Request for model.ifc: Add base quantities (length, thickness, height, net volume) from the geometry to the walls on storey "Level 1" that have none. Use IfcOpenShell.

First a look at what the model holds.

```python
import ifcopenshell
import ifcopenshell.util.element
import ifcopenshell.util.unit

model = ifcopenshell.open("model.ifc")
print(model.schema)
for unit_type in ("LENGTHUNIT", "AREAUNIT", "VOLUMEUNIT"):
    print(unit_type, ifcopenshell.util.unit.calculate_unit_scale(model, unit_type))
storey = next(s for s in model.by_type("IfcBuildingStorey") if s.Name == "Level 1")
walls = [e for e in ifcopenshell.util.element.get_decomposition(storey) if e.is_a("IfcWall")]
for e in sorted(walls, key=lambda e: e.id()):
    print(e.id(), e.is_a(), e.Name, list(ifcopenshell.util.element.get_psets(e, qtos_only=True)), sep=" | ")
```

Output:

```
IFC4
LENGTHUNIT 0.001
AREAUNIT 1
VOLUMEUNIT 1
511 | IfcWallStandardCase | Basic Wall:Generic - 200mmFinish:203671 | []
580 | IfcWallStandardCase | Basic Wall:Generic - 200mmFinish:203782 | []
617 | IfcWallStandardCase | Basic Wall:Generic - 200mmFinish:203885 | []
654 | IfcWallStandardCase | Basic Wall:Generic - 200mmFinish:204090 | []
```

```python
import ifcopenshell
import ifcopenshell.api.pset
import ifcopenshell.geom
import ifcopenshell.util.element
import ifcopenshell.util.shape
import ifcopenshell.util.unit

model = ifcopenshell.open("model.ifc")
unit_scale = ifcopenshell.util.unit.calculate_unit_scale(model)
volume_scale = ifcopenshell.util.unit.calculate_unit_scale(model, "VOLUMEUNIT")
settings = ifcopenshell.geom.settings()

storey = next(s for s in model.by_type("IfcBuildingStorey") if s.Name == "Level 1")
walls = [e for e in ifcopenshell.util.element.get_decomposition(storey) if e.is_a("IfcWall")]

for e in sorted(walls, key=lambda e: e.id()):
    if ifcopenshell.util.element.get_psets(e, qtos_only=True, should_inherit=False):
        continue
    # Geometry comes back in metres, in the element's own axes.
    shape = ifcopenshell.geom.create_shape(settings, e)
    values = {
        "Length": ifcopenshell.util.shape.get_x(shape.geometry) / unit_scale,
        "Width": ifcopenshell.util.shape.get_y(shape.geometry) / unit_scale,
        "Height": ifcopenshell.util.shape.get_z(shape.geometry) / unit_scale,
        "NetVolume": ifcopenshell.util.shape.get_volume(shape.geometry) / volume_scale,
    }
    qto = ifcopenshell.api.pset.add_qto(model, product=e, name="Qto_WallBaseQuantities")
    ifcopenshell.api.pset.edit_qto(model, qto=qto, properties=values)
    print(e.id(), {k: round(v, 3) for k, v in values.items()})

model.write("model_updated.ifc")
```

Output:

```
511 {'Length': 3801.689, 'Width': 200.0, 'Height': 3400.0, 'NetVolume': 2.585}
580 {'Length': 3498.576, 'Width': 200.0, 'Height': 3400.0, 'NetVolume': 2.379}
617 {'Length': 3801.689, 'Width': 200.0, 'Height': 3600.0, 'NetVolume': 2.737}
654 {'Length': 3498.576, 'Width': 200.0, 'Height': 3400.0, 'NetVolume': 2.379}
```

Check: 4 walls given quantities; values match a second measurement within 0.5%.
